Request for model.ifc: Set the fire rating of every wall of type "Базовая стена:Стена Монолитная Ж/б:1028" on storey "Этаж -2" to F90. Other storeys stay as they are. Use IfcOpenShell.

First a look at what the model holds.

```python
import ifcopenshell
import ifcopenshell.util.element

model = ifcopenshell.open("model.ifc")
print(model.schema)
storey = next(s for s in model.by_type("IfcBuildingStorey") if s.Name == "Этаж -2")
walls = [e for e in ifcopenshell.util.element.get_decomposition(storey) if e.is_a("IfcWall")]
seen = {}
for e in walls:
    element_type = ifcopenshell.util.element.get_type(e)
    key = (element_type.Name if element_type != e and element_type else None, ifcopenshell.util.element.get_pset(e, "Pset_WallCommon", "FireRating"))
    seen[key] = seen.get(key, 0) + 1
for (name, value), count in sorted(seen.items(), key=str):
    print(count, "x", name, "|", value)
```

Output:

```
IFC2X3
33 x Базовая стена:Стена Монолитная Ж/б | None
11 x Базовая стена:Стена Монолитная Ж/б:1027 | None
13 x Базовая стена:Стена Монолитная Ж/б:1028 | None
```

```python
import ifcopenshell
import ifcopenshell.api.pset
import ifcopenshell.util.element

model = ifcopenshell.open("model.ifc")

storey = next(s for s in model.by_type("IfcBuildingStorey") if s.Name == "Этаж -2")
walls = [e for e in ifcopenshell.util.element.get_decomposition(storey) if e.is_a("IfcWall")]

count = 0
for e in walls:
    element_type = ifcopenshell.util.element.get_type(e)
    if element_type in (None, e) or element_type.Name != "Базовая стена:Стена Монолитная Ж/б:1028":
        continue
    # add_pset returns the element's existing set when there is one.
    pset = ifcopenshell.api.pset.add_pset(model, product=e, name="Pset_WallCommon")
    ifcopenshell.api.pset.edit_pset(model, pset=pset, properties={"FireRating": "F90"})
    count += 1

print(count, "walls updated")

model.write("model_edited.ifc")
```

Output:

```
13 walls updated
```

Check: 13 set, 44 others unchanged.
